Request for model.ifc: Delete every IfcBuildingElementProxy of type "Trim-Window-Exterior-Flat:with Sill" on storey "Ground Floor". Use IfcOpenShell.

First a look at what the model holds.

```python
import ifcopenshell
import ifcopenshell.util.element

model = ifcopenshell.open("model.ifc")
print(model.schema)
storey = next(s for s in model.by_type("IfcBuildingStorey") if s.Name == "Ground Floor")
proxies = [e for e in ifcopenshell.util.element.get_decomposition(storey) if e.is_a("IfcBuildingElementProxy")]
seen = {}
for e in proxies:
    element_type = ifcopenshell.util.element.get_type(e)
    name = element_type.Name if element_type not in (None, e) else None
    seen[name] = seen.get(name, 0) + 1
for name, count in sorted(seen.items(), key=str):
    print(count, "x", name)
```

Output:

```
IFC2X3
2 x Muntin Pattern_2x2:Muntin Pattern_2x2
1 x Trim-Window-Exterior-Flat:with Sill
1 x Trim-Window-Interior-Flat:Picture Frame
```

```python
import ifcopenshell
import ifcopenshell.api.root
import ifcopenshell.util.element

model = ifcopenshell.open("model.ifc")

storey = next(s for s in model.by_type("IfcBuildingStorey") if s.Name == "Ground Floor")
proxies = [e for e in ifcopenshell.util.element.get_decomposition(storey) if e.is_a("IfcBuildingElementProxy")]
targets = [e for e in proxies if (t := ifcopenshell.util.element.get_type(e)) not in (None, e) and t.Name == "Trim-Window-Exterior-Flat:with Sill"]

for e in targets:
    ifcopenshell.api.root.remove_product(model, product=e)
print(len(targets), "removed")

model.write("model_rev.ifc")
```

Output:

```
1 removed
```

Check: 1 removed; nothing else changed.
